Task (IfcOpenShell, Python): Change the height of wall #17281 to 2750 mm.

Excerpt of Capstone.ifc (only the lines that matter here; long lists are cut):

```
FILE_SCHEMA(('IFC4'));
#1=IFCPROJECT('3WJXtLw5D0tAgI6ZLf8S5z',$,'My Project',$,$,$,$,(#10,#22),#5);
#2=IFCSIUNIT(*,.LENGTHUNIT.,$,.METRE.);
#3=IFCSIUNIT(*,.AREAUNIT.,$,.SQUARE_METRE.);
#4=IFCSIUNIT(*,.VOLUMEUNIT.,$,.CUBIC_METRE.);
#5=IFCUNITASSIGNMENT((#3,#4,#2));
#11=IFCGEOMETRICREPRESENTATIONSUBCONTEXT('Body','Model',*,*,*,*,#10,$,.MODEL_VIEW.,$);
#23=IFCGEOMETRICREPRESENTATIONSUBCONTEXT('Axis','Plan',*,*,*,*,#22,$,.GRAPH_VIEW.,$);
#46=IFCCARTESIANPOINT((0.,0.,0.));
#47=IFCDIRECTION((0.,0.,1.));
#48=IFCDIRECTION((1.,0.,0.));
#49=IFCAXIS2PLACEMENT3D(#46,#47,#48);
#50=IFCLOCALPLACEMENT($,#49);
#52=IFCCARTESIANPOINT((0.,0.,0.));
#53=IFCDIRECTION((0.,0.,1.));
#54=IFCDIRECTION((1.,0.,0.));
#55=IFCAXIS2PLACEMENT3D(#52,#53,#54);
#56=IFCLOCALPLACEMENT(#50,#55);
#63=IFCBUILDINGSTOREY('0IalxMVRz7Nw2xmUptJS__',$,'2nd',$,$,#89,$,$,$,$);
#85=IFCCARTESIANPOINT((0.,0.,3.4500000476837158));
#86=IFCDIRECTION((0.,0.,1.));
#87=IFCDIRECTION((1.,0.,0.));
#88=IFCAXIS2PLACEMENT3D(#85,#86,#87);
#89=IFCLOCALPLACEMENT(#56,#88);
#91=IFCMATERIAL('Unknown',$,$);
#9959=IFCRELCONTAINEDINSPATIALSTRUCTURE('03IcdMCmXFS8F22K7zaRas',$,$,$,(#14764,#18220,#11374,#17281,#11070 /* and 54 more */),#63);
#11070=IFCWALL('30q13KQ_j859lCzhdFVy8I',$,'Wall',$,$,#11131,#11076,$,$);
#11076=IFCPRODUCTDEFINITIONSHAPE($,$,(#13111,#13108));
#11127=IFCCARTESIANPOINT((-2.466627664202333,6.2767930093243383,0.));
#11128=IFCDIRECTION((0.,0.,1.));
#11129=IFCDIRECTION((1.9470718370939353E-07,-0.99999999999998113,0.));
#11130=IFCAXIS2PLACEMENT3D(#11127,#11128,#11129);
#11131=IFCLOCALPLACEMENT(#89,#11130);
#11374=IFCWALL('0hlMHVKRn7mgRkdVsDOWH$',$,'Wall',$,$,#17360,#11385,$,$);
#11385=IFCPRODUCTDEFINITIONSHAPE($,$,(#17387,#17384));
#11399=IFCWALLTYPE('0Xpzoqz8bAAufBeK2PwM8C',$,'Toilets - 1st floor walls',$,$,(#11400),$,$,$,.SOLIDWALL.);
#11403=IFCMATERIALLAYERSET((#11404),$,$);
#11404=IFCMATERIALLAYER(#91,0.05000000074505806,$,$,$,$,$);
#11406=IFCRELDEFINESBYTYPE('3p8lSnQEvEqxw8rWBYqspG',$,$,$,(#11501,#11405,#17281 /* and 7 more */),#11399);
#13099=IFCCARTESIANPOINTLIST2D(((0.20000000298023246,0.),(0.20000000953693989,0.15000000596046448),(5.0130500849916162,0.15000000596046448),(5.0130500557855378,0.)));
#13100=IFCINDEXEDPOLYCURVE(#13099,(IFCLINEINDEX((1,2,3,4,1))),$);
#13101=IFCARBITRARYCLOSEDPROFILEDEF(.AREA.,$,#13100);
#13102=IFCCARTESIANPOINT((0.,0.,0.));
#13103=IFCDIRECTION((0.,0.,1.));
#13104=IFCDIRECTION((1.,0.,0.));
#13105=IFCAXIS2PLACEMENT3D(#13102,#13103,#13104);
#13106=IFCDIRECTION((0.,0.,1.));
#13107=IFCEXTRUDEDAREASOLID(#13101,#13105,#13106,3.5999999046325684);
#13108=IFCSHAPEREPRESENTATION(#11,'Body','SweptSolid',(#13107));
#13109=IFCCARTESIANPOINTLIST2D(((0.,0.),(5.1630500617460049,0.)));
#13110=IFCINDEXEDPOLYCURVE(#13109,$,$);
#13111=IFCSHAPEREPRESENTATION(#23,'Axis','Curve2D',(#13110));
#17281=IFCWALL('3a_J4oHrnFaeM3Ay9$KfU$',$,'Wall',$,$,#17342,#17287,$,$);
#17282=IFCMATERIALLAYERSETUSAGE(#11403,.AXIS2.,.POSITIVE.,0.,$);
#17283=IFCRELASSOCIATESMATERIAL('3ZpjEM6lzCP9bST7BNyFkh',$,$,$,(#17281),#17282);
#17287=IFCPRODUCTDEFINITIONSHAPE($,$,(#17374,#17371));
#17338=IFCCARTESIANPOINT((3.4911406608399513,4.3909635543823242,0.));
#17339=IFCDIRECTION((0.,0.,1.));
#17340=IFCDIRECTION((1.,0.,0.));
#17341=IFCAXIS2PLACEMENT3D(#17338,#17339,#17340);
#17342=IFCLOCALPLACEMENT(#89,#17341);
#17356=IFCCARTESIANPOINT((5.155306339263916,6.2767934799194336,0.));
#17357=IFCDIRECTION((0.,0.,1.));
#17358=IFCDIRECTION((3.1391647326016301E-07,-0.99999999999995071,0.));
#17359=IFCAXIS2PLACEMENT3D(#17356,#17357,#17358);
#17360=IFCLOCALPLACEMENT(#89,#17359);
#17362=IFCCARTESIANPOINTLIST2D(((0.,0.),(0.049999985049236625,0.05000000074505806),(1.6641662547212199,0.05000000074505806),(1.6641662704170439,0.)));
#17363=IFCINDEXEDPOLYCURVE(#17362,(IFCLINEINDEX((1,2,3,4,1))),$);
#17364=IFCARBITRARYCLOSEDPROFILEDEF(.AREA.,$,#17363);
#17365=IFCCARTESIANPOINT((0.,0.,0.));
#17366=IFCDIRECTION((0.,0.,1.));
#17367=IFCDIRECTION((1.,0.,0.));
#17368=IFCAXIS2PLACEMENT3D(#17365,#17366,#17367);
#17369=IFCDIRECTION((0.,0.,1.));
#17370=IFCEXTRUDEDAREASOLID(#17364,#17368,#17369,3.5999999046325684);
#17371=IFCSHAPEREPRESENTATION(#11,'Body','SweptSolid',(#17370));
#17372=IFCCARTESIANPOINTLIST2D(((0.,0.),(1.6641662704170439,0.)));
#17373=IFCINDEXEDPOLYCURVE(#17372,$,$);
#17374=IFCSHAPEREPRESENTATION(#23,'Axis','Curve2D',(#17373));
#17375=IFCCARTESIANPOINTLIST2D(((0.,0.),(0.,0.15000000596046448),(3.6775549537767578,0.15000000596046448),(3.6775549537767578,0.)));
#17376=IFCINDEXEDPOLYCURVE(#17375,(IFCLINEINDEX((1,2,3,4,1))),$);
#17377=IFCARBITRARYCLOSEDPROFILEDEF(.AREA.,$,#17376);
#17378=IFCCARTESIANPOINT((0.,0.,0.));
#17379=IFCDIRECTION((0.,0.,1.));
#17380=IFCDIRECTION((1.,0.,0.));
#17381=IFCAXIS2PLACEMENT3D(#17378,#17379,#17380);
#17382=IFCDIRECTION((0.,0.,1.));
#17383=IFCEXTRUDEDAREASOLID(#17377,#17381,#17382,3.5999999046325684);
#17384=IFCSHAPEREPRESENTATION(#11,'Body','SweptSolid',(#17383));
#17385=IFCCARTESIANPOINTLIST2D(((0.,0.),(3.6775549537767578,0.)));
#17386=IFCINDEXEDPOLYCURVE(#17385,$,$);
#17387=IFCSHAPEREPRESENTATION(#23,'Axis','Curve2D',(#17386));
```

```python
import ifcopenshell
import ifcopenshell.geom
import ifcopenshell.util.representation
import ifcopenshell.util.shape
import ifcopenshell.util.unit

model = ifcopenshell.open("Capstone.ifc")
unit_scale = ifcopenshell.util.unit.calculate_unit_scale(model)
settings = ifcopenshell.geom.settings()


def volume(element):
    """Net volume in cubic metres, openings subtracted."""
    shape = ifcopenshell.geom.create_shape(settings, element)
    return ifcopenshell.util.shape.get_volume(shape.geometry)


wall = model.by_guid("3a_J4oHrnFaeM3Ay9$KfU$")
before = volume(wall)

body = ifcopenshell.util.representation.get_representation(wall, "Model", "Body")
solid = body.Items[0]
old_height = solid.Depth
solid.Depth = 2.75 / unit_scale
after = volume(wall)

print(f"height {old_height:g} -> {solid.Depth:g}, volume {before:.3f} -> {after:.3f} m3")

model.write("Capstone_edited.ifc")
```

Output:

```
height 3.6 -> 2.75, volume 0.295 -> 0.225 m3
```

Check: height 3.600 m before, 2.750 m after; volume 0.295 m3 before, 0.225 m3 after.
